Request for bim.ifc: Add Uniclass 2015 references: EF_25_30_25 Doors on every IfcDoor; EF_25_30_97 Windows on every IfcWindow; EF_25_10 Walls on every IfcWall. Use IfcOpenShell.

First a look at what the model holds.

```python
import ifcopenshell

model = ifcopenshell.open("bim.ifc")
print(model.schema)
print("classifications:", [c.Name for c in model.by_type("IfcClassification")])
for ifc_class in ("IfcDoor", "IfcRoof", "IfcStair", "IfcWall", "IfcWindow"):
    print(ifc_class, len(model.by_type(ifc_class)))
```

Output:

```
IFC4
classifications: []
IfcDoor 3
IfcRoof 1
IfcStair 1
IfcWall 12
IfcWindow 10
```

```python
import ifcopenshell
import ifcopenshell.api.classification

model = ifcopenshell.open("bim.ifc")

system = ifcopenshell.api.classification.add_classification(model, classification="Uniclass 2015")

codes = {
    "IfcDoor": ("EF_25_30_25", "Doors"),
    "IfcWindow": ("EF_25_30_97", "Windows"),
    "IfcWall": ("EF_25_10", "Walls"),
}
for ifc_class, (code, name) in codes.items():
    products = model.by_type(ifc_class)
    ifcopenshell.api.classification.add_reference(
        model, products=products, classification=system, identification=code, name=name
    )
    print(code, len(products))

model.write("bim_edited.ifc")
```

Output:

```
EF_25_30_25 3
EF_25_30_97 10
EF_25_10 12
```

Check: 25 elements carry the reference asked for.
